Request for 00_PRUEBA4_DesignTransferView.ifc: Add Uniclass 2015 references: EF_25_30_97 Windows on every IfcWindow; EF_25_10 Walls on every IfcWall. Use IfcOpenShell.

First a look at what the model holds.

```python
import ifcopenshell

model = ifcopenshell.open("00_PRUEBA4_DesignTransferView.ifc")
print(model.schema)
print("classifications:", [c.Name for c in model.by_type("IfcClassification")])
for ifc_class in ("IfcDoor", "IfcRoof", "IfcStair", "IfcWall", "IfcWindow"):
    print(ifc_class, len(model.by_type(ifc_class)))
```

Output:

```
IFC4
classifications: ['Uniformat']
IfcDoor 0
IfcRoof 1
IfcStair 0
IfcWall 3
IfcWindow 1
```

```python
import ifcopenshell
import ifcopenshell.api.classification

model = ifcopenshell.open("00_PRUEBA4_DesignTransferView.ifc")

system = ifcopenshell.api.classification.add_classification(model, classification="Uniclass 2015")

codes = {
    "IfcWindow": ("EF_25_30_97", "Windows"),
    "IfcWall": ("EF_25_10", "Walls"),
}
for ifc_class, (code, name) in codes.items():
    products = model.by_type(ifc_class)
    ifcopenshell.api.classification.add_reference(
        model, products=products, classification=system, identification=code, name=name
    )
    print(code, len(products))

model.write("00_PRUEBA4_DesignTransferView-out.ifc")
```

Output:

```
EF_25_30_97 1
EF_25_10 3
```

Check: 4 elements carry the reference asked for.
